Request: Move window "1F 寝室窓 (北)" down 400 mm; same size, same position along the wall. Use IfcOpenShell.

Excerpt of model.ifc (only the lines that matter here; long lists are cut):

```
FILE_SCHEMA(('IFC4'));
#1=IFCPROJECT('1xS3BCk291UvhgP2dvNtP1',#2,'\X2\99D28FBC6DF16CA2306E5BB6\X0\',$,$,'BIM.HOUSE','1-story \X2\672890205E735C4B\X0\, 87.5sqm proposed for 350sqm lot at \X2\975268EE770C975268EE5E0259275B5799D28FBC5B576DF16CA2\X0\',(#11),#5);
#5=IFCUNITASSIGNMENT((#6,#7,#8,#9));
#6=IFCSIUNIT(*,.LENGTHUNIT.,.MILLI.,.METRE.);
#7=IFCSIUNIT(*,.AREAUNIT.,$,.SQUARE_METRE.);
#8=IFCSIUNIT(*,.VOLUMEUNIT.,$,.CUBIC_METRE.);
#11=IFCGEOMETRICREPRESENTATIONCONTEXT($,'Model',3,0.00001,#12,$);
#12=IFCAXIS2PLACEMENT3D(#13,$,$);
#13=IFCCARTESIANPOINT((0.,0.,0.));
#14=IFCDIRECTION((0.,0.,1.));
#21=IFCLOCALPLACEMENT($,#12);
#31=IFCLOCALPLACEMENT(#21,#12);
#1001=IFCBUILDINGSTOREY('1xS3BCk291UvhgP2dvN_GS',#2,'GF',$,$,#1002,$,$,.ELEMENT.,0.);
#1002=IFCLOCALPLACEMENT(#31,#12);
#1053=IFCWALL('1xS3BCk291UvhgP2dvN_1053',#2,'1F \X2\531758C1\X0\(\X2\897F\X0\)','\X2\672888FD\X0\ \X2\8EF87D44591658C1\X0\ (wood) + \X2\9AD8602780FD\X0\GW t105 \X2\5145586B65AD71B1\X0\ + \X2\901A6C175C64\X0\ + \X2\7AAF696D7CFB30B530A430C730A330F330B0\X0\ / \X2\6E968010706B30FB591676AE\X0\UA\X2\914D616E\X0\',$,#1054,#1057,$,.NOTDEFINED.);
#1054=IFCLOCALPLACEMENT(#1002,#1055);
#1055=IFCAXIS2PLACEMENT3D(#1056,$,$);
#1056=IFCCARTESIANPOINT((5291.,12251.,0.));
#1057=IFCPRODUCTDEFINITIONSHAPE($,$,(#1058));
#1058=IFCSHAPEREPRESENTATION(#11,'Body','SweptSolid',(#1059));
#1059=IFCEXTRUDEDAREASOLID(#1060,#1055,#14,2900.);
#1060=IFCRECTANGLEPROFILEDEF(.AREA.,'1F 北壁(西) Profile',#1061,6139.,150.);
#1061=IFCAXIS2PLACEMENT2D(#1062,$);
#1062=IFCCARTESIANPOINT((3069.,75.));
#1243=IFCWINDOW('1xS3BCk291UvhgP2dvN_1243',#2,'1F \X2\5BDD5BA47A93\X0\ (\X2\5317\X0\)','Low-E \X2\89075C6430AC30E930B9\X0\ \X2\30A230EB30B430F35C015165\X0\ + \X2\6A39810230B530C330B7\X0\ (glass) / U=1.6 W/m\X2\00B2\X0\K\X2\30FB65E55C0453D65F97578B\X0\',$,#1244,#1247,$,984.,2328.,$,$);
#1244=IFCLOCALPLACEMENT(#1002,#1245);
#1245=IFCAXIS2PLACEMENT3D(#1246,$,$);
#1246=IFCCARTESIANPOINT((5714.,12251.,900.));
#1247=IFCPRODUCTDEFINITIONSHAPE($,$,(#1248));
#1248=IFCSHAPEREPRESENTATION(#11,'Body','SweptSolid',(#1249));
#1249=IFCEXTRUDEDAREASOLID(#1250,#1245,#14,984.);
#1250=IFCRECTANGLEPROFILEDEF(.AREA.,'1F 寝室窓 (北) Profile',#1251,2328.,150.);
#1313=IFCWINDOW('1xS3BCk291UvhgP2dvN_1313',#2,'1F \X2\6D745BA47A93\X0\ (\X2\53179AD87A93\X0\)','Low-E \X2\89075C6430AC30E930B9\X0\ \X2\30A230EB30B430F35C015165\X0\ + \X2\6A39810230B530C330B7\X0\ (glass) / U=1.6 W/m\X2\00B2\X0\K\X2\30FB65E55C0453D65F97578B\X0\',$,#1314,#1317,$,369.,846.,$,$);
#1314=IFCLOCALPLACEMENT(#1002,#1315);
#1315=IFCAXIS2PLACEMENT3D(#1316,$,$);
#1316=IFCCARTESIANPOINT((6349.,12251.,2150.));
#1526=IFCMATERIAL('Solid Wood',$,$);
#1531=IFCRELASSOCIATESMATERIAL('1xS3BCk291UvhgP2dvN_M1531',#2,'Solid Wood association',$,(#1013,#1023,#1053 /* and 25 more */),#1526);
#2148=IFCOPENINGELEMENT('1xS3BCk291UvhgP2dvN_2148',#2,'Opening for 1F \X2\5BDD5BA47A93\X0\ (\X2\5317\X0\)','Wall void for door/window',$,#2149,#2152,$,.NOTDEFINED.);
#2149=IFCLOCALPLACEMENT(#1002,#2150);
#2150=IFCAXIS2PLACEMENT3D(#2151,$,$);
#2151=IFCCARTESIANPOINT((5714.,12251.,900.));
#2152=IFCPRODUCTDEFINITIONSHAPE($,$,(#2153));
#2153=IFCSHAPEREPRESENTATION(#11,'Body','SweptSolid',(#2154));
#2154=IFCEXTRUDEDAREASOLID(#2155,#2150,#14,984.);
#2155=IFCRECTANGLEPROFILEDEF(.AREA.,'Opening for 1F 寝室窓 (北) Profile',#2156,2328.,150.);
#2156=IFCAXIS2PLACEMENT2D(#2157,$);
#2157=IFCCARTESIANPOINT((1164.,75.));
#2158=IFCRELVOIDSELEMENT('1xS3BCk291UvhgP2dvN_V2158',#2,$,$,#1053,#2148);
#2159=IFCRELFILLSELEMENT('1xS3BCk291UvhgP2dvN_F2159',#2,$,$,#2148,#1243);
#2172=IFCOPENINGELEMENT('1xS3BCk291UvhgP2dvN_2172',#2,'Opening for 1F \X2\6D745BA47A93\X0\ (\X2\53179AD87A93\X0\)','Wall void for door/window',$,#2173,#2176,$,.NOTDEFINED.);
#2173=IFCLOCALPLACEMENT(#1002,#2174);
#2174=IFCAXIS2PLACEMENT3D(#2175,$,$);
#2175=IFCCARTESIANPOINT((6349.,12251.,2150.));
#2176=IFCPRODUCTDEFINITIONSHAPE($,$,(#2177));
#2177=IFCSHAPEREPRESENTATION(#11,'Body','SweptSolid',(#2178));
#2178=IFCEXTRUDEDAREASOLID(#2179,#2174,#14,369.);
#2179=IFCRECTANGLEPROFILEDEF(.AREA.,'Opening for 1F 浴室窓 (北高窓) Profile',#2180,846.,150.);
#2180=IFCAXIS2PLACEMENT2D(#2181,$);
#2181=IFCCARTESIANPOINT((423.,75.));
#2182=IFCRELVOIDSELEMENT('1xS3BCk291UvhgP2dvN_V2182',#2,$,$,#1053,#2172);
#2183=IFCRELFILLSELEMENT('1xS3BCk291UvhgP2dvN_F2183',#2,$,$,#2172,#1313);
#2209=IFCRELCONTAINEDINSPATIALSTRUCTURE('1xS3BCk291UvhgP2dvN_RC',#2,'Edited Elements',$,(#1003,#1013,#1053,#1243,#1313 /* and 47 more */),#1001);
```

```python
import numpy as np
import ifcopenshell
import ifcopenshell.api.geometry
import ifcopenshell.util.placement
import ifcopenshell.util.unit

model = ifcopenshell.open("model.ifc")
unit_scale = ifcopenshell.util.unit.calculate_unit_scale(model)

window = model.by_guid("1xS3BCk291UvhgP2dvN_1243")
opening = window.FillsVoids[0].RelatingOpeningElement
dz = -0.4 / unit_scale

shift = np.array([0.0, 0.0, dz])
# The window is not placed relative to its opening, so move both.
for product in (opening, window):
    matrix = ifcopenshell.util.placement.get_local_placement(product.ObjectPlacement)
    matrix[:3, 3] += shift
    ifcopenshell.api.geometry.edit_object_placement(model, product=product, matrix=matrix, is_si=False)

print(f"moved by {dz * unit_scale:+.3f} m")

model.write("model-out.ifc")
```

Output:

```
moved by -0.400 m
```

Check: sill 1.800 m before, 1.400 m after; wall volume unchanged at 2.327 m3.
